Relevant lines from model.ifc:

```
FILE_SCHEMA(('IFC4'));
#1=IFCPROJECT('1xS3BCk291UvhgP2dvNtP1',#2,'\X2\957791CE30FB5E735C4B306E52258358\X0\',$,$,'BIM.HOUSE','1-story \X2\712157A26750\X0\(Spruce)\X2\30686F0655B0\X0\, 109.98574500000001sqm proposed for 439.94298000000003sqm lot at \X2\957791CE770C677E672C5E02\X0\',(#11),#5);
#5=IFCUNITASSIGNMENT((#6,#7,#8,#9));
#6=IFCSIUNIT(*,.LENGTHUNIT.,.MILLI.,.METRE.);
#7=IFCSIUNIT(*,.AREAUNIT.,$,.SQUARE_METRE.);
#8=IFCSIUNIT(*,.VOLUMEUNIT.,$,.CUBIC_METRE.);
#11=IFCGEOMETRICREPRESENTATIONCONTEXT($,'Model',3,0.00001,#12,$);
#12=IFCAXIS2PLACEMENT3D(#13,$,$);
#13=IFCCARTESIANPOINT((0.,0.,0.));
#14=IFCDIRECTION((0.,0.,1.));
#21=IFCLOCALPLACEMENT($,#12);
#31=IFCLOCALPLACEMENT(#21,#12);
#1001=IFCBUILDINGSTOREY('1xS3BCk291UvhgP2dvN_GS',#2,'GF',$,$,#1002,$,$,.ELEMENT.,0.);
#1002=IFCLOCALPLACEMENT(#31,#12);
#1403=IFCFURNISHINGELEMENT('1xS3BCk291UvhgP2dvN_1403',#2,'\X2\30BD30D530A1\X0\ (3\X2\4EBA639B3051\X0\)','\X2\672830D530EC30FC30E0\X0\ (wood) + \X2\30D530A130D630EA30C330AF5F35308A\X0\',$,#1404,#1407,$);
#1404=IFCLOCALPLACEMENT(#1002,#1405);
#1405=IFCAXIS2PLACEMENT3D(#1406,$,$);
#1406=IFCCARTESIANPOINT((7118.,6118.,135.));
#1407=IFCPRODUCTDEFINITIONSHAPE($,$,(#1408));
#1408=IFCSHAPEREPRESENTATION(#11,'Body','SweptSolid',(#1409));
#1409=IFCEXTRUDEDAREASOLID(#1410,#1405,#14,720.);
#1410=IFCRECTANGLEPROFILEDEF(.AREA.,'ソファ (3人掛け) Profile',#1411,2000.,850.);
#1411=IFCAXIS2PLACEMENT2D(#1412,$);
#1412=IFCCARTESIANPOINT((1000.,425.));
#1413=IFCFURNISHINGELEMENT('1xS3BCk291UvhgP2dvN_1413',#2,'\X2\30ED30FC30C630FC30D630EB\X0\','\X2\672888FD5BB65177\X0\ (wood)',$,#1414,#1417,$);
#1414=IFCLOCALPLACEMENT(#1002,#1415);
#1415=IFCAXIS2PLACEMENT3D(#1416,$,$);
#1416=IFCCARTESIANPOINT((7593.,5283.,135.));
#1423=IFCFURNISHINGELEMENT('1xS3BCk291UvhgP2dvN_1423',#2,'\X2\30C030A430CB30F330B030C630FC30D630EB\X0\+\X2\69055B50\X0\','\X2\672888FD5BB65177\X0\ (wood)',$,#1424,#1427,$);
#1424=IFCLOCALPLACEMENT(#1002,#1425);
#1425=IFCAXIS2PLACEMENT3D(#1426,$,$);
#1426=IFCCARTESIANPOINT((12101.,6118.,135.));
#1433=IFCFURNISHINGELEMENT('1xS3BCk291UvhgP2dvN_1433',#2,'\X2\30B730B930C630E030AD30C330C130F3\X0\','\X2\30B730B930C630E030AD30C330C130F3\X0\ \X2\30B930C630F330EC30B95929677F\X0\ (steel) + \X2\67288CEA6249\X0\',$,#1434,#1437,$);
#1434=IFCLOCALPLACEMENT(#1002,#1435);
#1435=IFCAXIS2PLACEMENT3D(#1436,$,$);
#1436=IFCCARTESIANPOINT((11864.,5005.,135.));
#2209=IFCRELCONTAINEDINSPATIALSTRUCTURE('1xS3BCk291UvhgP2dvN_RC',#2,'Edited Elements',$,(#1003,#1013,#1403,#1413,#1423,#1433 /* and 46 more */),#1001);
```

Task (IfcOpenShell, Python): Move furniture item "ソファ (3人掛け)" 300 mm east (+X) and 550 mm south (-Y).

```python
import ifcopenshell
import ifcopenshell.api.geometry
import ifcopenshell.util.placement

model = ifcopenshell.open("model.ifc")

item = model.by_guid("1xS3BCk291UvhgP2dvN_1403")
matrix = ifcopenshell.util.placement.get_local_placement(item.ObjectPlacement)
matrix[0, 3] += 300.0
matrix[1, 3] -= 550.0
ifcopenshell.api.geometry.edit_object_placement(model, product=item, matrix=matrix, is_si=False)

print(ifcopenshell.util.placement.get_local_placement(item.ObjectPlacement).round(3) + 0.0)

model.write("model_v2.ifc")
```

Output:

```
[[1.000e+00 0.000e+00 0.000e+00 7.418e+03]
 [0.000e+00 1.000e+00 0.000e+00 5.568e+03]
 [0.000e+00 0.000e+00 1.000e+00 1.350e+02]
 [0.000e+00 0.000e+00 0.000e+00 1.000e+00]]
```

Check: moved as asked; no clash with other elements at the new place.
